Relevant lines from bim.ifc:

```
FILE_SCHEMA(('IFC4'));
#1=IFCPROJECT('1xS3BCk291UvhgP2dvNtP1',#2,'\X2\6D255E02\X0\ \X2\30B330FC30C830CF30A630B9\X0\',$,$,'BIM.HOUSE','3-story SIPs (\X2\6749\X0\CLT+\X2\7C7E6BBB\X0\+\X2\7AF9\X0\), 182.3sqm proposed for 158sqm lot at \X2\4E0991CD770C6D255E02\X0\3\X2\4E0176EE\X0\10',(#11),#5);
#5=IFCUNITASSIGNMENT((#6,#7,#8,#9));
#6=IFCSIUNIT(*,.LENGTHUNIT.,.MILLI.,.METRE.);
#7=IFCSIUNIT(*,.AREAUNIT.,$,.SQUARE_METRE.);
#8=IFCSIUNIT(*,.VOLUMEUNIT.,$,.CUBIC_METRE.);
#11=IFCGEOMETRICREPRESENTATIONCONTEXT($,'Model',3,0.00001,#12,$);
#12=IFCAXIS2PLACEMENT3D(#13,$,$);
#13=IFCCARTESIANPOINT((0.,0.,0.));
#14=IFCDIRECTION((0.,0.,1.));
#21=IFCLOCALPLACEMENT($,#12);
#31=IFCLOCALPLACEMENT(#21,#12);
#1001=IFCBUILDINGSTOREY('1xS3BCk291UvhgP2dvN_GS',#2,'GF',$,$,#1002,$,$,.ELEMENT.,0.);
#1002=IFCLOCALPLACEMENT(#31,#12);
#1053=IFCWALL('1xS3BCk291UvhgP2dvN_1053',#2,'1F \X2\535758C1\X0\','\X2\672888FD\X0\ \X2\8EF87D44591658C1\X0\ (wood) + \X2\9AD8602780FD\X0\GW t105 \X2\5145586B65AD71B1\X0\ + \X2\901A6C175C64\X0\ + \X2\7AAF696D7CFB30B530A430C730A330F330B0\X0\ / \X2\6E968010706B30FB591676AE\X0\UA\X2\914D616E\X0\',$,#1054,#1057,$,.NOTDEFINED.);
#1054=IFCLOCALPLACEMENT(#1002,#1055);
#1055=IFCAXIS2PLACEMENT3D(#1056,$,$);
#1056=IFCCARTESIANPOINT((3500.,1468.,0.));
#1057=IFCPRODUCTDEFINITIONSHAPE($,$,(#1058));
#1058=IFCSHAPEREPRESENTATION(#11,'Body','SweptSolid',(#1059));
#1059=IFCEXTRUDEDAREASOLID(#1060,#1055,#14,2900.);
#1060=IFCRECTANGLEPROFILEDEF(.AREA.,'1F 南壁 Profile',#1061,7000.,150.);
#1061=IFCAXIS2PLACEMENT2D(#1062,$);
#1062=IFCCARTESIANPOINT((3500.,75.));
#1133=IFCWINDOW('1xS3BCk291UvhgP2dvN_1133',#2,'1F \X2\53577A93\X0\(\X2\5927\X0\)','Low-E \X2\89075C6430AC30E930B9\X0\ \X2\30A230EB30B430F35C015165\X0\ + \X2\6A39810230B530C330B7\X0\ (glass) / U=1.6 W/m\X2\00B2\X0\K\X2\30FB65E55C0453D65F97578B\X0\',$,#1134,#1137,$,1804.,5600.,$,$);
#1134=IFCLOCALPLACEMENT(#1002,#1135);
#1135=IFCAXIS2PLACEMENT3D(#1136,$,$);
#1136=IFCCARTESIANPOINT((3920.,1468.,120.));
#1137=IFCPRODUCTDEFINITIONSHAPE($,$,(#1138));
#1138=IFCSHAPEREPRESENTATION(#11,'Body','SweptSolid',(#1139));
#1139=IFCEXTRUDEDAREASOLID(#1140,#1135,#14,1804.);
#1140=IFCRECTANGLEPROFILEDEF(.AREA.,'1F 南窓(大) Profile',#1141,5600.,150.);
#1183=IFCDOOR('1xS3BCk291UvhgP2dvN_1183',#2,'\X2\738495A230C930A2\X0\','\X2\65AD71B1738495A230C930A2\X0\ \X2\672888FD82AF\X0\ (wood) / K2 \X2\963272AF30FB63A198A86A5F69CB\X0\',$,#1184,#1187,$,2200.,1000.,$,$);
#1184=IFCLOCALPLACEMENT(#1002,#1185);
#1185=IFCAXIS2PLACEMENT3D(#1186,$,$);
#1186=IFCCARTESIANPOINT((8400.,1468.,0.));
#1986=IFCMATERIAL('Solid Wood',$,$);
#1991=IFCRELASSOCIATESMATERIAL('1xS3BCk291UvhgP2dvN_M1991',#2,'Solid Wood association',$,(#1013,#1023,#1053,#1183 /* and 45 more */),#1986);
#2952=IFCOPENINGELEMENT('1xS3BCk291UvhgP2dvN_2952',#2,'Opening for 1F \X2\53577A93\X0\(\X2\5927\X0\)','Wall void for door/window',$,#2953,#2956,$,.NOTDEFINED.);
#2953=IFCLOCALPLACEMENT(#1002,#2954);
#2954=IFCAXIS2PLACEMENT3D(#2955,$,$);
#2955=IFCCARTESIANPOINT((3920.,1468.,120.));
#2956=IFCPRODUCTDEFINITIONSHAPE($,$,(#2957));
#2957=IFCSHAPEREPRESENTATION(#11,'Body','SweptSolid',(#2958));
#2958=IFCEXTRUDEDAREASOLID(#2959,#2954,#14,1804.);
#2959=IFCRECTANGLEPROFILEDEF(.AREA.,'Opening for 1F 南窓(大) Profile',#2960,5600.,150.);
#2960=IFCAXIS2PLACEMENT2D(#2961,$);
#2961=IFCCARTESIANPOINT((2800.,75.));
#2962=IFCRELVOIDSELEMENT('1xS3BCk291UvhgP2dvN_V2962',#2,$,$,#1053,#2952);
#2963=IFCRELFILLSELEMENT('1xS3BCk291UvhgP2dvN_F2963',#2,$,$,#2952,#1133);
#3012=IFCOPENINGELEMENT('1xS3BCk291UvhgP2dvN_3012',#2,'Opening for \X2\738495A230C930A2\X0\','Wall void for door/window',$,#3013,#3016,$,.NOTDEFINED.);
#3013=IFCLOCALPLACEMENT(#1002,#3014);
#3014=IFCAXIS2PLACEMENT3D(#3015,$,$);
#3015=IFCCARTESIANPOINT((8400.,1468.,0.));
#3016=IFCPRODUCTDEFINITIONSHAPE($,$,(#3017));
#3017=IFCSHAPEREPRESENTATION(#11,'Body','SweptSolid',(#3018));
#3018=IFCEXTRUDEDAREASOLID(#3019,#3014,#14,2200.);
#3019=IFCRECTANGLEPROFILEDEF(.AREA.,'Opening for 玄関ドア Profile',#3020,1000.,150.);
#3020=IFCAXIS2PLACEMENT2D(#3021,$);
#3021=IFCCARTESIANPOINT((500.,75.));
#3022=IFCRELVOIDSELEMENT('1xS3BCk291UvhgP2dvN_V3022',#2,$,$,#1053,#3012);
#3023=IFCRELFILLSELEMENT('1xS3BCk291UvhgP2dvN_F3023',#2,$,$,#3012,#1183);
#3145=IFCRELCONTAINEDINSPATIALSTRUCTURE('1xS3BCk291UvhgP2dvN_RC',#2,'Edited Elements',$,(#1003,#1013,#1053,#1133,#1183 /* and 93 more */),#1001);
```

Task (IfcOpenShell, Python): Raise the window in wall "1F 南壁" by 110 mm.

```python
import numpy as np
import ifcopenshell
import ifcopenshell.api.geometry
import ifcopenshell.util.placement
import ifcopenshell.util.unit

model = ifcopenshell.open("bim.ifc")
unit_scale = ifcopenshell.util.unit.calculate_unit_scale(model)

window = model.by_guid("1xS3BCk291UvhgP2dvN_1133")
opening = window.FillsVoids[0].RelatingOpeningElement
dz = 110.0

shift = np.array([0.0, 0.0, dz])
# The window is not placed relative to its opening, so move both.
for product in (opening, window):
    matrix = ifcopenshell.util.placement.get_local_placement(product.ObjectPlacement)
    matrix[:3, 3] += shift
    ifcopenshell.api.geometry.edit_object_placement(model, product=product, matrix=matrix, is_si=False)

print(f"moved by {dz * unit_scale:+.3f} m")

model.write("bim_rev.ifc")
```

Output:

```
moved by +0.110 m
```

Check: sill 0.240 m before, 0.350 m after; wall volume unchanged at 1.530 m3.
